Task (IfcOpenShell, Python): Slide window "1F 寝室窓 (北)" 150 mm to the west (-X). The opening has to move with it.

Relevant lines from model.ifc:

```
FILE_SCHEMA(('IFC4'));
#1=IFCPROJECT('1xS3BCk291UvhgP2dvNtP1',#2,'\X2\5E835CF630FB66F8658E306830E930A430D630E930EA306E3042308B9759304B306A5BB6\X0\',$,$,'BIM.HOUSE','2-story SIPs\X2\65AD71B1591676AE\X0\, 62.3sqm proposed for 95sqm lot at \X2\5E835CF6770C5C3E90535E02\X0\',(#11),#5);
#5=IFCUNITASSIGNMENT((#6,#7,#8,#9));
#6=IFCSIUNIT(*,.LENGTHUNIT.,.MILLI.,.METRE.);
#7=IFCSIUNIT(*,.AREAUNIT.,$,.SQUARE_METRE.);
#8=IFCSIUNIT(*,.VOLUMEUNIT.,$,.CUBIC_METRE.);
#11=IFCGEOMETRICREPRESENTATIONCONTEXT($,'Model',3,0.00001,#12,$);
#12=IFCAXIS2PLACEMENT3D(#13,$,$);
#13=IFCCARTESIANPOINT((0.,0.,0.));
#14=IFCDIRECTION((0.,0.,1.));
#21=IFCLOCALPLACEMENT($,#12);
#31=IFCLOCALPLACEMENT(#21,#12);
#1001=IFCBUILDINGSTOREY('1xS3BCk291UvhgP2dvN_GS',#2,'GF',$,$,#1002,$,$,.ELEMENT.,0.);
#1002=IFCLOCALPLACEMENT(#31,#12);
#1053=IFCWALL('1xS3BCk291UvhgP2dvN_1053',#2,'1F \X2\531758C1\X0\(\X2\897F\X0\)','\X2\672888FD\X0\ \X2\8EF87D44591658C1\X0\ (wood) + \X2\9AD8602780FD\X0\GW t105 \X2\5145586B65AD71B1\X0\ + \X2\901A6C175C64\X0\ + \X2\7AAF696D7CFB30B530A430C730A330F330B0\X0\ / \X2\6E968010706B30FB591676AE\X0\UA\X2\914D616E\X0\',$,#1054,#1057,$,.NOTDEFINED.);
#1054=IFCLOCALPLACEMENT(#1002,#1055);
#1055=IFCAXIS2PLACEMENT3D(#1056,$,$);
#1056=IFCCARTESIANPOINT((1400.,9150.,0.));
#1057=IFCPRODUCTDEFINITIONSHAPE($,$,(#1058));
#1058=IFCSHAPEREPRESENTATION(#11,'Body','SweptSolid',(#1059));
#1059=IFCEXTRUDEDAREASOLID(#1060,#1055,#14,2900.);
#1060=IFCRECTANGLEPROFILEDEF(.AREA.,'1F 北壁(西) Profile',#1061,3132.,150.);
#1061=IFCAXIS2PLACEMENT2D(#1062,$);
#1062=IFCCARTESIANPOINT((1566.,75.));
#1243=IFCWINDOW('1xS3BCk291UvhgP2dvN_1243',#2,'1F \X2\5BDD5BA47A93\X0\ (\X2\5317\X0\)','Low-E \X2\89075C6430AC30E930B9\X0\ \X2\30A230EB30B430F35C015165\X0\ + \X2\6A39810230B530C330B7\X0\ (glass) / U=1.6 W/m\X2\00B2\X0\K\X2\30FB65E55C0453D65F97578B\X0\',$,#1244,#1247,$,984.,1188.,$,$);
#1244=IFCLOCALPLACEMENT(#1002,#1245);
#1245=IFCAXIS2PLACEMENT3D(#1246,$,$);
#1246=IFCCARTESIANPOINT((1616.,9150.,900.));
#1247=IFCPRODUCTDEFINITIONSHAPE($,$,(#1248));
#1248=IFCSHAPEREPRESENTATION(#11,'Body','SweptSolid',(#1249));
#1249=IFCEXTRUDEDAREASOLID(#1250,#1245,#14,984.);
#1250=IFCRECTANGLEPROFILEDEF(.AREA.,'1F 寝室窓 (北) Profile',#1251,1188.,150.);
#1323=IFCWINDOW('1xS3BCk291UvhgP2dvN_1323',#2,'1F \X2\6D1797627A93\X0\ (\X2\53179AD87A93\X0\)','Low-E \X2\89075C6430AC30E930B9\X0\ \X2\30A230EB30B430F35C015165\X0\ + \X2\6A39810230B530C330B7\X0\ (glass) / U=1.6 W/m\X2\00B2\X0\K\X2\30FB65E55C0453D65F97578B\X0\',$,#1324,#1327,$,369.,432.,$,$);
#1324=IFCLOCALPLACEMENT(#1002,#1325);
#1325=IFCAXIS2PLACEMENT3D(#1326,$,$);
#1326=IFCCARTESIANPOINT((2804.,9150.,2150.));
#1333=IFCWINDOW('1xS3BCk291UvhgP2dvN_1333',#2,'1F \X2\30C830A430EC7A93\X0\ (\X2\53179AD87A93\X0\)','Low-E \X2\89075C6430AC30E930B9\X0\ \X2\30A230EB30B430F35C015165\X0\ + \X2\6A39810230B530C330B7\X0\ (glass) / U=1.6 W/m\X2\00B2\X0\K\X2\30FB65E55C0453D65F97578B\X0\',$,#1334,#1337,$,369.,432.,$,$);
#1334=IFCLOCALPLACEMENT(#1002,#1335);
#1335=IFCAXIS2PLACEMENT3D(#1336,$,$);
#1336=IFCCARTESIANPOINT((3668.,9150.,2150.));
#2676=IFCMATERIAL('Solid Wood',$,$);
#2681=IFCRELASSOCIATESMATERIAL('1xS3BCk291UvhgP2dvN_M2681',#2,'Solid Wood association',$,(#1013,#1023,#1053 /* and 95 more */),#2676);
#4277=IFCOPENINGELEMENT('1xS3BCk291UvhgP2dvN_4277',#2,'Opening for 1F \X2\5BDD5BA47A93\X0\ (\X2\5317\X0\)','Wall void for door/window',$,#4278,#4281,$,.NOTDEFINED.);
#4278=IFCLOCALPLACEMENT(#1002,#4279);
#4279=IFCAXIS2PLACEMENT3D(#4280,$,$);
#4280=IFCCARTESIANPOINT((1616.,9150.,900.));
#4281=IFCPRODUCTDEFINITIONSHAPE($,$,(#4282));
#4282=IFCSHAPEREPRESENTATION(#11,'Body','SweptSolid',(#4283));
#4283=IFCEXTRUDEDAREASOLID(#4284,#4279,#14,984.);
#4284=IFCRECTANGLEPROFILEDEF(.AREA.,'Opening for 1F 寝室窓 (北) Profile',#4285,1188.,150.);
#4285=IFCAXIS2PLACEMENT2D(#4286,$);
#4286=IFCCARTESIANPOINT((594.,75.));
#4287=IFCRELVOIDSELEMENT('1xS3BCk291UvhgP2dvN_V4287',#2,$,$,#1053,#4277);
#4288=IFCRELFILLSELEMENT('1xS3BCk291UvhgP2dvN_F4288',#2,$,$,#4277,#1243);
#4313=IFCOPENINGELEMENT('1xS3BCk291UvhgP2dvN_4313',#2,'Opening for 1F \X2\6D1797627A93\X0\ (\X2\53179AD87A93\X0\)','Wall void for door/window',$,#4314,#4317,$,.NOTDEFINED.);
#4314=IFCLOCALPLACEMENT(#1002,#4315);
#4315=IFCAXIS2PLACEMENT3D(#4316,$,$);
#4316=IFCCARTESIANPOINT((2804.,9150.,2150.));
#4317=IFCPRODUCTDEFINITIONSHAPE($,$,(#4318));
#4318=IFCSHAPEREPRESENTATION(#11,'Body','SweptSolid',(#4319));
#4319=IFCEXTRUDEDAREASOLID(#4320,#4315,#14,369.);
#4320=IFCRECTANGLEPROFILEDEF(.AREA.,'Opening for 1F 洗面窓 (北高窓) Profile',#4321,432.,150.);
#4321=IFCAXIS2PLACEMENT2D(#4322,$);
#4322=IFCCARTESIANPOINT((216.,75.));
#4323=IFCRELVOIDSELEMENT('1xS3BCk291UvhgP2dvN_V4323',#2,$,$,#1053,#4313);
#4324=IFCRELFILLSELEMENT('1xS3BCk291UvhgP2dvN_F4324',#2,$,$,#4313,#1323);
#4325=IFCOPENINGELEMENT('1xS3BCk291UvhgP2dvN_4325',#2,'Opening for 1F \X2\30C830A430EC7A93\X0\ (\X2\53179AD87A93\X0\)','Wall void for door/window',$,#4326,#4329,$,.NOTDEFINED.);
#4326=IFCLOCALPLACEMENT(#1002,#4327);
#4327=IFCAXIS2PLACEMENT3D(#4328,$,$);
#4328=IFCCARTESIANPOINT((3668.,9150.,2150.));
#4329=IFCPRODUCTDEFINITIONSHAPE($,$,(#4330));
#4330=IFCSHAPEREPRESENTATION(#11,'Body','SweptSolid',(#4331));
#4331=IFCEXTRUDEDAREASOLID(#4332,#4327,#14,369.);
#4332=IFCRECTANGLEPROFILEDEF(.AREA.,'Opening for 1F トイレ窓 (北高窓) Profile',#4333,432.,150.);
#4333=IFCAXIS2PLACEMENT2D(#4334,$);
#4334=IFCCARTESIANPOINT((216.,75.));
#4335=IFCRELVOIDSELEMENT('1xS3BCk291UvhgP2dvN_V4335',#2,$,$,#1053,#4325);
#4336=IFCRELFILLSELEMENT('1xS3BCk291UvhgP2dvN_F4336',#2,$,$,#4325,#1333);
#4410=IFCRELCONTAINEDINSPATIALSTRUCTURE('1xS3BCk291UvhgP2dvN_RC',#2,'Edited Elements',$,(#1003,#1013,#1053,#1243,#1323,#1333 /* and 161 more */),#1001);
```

```python
import ifcopenshell
import ifcopenshell.api.geometry
import ifcopenshell.util.placement

model = ifcopenshell.open("model.ifc")

window = model.by_id(1243)
opening = window.FillsVoids[0].RelatingOpeningElement
wall = opening.VoidsElements[0].RelatingBuildingElement

wall_matrix = ifcopenshell.util.placement.get_local_placement(wall.ObjectPlacement)
shift = wall_matrix[:3, 0] * -150.0
before = ifcopenshell.util.placement.get_local_placement(window.ObjectPlacement)[:3, 3].copy()

# The window is not placed relative to its opening, so move both.
for product in (opening, window):
    matrix = ifcopenshell.util.placement.get_local_placement(product.ObjectPlacement)
    matrix[:3, 3] += shift
    ifcopenshell.api.geometry.edit_object_placement(model, product=product, matrix=matrix, is_si=False)

after = ifcopenshell.util.placement.get_local_placement(window.ObjectPlacement)[:3, 3]
print("window moved by", (after - before).round(3) + 0.0)

model.write("model_rev.ifc")
```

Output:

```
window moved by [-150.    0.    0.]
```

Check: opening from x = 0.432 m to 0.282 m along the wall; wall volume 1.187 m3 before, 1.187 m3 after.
